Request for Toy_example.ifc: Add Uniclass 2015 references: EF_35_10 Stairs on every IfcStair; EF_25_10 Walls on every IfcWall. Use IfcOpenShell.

First a look at what the model holds.

```python
import ifcopenshell

model = ifcopenshell.open("Toy_example.ifc")
print(model.schema)
print("classifications:", [c.Name for c in model.by_type("IfcClassification")])
for ifc_class in ("IfcDoor", "IfcRoof", "IfcStair", "IfcWall", "IfcWindow"):
    print(ifc_class, len(model.by_type(ifc_class)))
```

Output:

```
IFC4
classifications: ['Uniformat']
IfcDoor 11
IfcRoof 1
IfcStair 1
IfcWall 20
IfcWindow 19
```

```python
import ifcopenshell
import ifcopenshell.api.classification

model = ifcopenshell.open("Toy_example.ifc")

system = ifcopenshell.api.classification.add_classification(model, classification="Uniclass 2015")

codes = {
    "IfcStair": ("EF_35_10", "Stairs"),
    "IfcWall": ("EF_25_10", "Walls"),
}
for ifc_class, (code, name) in codes.items():
    products = model.by_type(ifc_class)
    ifcopenshell.api.classification.add_reference(
        model, products=products, classification=system, identification=code, name=name
    )
    print(code, len(products))

model.write("Toy_example_v2.ifc")
```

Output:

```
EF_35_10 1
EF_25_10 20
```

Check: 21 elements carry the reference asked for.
